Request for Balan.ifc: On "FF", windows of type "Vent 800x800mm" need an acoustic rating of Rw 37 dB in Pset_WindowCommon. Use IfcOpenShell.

First a look at what the model holds.

```python
import ifcopenshell
import ifcopenshell.util.element

model = ifcopenshell.open("Balan.ifc")
print(model.schema)
storey = next(s for s in model.by_type("IfcBuildingStorey") if s.Name == "FF")
windows = [e for e in ifcopenshell.util.element.get_decomposition(storey) if e.is_a("IfcWindow")]
seen = {}
for e in windows:
    element_type = ifcopenshell.util.element.get_type(e)
    key = (element_type.Name if element_type != e and element_type else None, ifcopenshell.util.element.get_pset(e, "Pset_WindowCommon", "AcousticRating"))
    seen[key] = seen.get(key, 0) + 1
for (name, value), count in sorted(seen.items(), key=str):
    print(count, "x", name, "|", value)
```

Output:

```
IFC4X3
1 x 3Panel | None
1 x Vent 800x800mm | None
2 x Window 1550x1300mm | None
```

```python
import ifcopenshell
import ifcopenshell.api.pset
import ifcopenshell.util.element

model = ifcopenshell.open("Balan.ifc")

storey = next(s for s in model.by_type("IfcBuildingStorey") if s.Name == "FF")
windows = [e for e in ifcopenshell.util.element.get_decomposition(storey) if e.is_a("IfcWindow")]

count = 0
for e in windows:
    element_type = ifcopenshell.util.element.get_type(e)
    if element_type in (None, e) or element_type.Name != "Vent 800x800mm":
        continue
    # add_pset returns the element's existing set when there is one.
    pset = ifcopenshell.api.pset.add_pset(model, product=e, name="Pset_WindowCommon")
    ifcopenshell.api.pset.edit_pset(model, pset=pset, properties={"AcousticRating": "Rw 37 dB"})
    count += 1

print(count, "windows updated")

model.write("Balan_edited.ifc")
```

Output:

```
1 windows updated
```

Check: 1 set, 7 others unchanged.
